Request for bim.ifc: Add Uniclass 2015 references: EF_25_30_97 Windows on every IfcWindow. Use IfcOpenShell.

First a look at what the model holds.

```python
import ifcopenshell

model = ifcopenshell.open("bim.ifc")
print(model.schema)
print("classifications:", [c.Name for c in model.by_type("IfcClassification")])
for ifc_class in ("IfcDoor", "IfcRoof", "IfcStair", "IfcWall", "IfcWindow"):
    print(ifc_class, len(model.by_type(ifc_class)))
```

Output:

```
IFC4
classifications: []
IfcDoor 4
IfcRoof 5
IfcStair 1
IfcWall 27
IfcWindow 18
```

```python
import ifcopenshell
import ifcopenshell.api.classification

model = ifcopenshell.open("bim.ifc")

system = ifcopenshell.api.classification.add_classification(model, classification="Uniclass 2015")

codes = {
    "IfcWindow": ("EF_25_30_97", "Windows"),
}
for ifc_class, (code, name) in codes.items():
    products = model.by_type(ifc_class)
    ifcopenshell.api.classification.add_reference(
        model, products=products, classification=system, identification=code, name=name
    )
    print(code, len(products))

model.write("bim_v2.ifc")
```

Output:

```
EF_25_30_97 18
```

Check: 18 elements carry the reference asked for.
